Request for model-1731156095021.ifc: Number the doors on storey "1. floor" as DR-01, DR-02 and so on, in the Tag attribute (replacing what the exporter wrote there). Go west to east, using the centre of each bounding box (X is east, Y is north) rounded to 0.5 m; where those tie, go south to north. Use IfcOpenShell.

First a look at what the model holds.

```python
import ifcopenshell
import ifcopenshell.util.element
import ifcopenshell.util.placement

model = ifcopenshell.open("model-1731156095021.ifc")
print(model.schema)
storey = next(s for s in model.by_type("IfcBuildingStorey") if s.Name == "1. floor")
doors = [e for e in ifcopenshell.util.element.get_decomposition(storey) if e.is_a("IfcDoor")]
for e in sorted(doors, key=lambda e: e.id()):
    origin = ifcopenshell.util.placement.get_local_placement(e.ObjectPlacement)[:3, 3]
    print(e.id(), e.Tag, e.Name, origin.round(2) + 0.0, sep=" | ")
```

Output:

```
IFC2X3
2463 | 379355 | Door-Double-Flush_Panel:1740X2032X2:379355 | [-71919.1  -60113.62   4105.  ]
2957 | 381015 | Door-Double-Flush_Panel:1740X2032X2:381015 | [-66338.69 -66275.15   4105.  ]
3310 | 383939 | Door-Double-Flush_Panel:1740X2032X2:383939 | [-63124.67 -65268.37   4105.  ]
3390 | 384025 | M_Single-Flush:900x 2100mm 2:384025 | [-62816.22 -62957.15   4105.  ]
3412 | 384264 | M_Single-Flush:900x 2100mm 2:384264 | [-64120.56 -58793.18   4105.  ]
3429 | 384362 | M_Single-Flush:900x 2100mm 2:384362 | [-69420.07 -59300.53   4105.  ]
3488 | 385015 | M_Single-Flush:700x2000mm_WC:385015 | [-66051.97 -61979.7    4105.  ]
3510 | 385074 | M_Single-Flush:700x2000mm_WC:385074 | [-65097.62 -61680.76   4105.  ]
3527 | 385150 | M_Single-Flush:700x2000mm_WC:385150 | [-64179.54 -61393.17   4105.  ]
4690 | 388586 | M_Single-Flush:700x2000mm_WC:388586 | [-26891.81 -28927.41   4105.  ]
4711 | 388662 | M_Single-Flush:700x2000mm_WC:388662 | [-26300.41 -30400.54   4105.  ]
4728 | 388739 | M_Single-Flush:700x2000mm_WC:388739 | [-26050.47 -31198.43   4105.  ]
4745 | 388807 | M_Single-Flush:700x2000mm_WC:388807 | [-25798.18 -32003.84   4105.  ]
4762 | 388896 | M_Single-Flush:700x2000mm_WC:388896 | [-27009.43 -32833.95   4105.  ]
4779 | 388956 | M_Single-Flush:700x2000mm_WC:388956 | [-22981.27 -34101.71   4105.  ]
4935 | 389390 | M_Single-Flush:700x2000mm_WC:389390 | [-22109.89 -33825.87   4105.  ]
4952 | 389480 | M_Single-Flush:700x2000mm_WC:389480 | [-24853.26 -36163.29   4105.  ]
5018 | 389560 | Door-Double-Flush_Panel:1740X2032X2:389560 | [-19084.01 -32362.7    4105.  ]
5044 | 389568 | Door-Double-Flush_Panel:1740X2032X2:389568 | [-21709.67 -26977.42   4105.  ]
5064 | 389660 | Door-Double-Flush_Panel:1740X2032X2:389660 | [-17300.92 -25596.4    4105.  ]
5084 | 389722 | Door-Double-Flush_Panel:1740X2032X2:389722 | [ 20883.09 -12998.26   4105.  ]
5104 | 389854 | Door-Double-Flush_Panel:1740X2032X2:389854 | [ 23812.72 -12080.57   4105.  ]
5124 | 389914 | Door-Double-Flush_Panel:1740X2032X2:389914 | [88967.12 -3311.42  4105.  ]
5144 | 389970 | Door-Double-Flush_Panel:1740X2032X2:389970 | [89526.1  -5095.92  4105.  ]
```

```python
import ifcopenshell
import ifcopenshell.geom
import ifcopenshell.util.element
import ifcopenshell.util.shape

model = ifcopenshell.open("model-1731156095021.ifc")
settings = ifcopenshell.geom.settings()
settings.set("use-world-coords", True)


def centre(element):
    shape = ifcopenshell.geom.create_shape(settings, element)
    return ifcopenshell.util.shape.get_bbox_centroid(shape.geometry)


storey = next(s for s in model.by_type("IfcBuildingStorey") if s.Name == "1. floor")
doors = [e for e in ifcopenshell.util.element.get_decomposition(storey) if e.is_a("IfcDoor")]

# Insertion points can sit at a corner or the storey origin, so sort by the geometry (in metres).
centres = {e: centre(e) for e in doors}
doors.sort(key=lambda e: (round(centres[e][0] / 0.5), centres[e][1]))

for i, e in enumerate(doors, start=1):
    number = f"DR-{i:02d}"
    e.Tag = number
    print(e.id(), number)

model.write("model-1731156095021_edited.ifc")
```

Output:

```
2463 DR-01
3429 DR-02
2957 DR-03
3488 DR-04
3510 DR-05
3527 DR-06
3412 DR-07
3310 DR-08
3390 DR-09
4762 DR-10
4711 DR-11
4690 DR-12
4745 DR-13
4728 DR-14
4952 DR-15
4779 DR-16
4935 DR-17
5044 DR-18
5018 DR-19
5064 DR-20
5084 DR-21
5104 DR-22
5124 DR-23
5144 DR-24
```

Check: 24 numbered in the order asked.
